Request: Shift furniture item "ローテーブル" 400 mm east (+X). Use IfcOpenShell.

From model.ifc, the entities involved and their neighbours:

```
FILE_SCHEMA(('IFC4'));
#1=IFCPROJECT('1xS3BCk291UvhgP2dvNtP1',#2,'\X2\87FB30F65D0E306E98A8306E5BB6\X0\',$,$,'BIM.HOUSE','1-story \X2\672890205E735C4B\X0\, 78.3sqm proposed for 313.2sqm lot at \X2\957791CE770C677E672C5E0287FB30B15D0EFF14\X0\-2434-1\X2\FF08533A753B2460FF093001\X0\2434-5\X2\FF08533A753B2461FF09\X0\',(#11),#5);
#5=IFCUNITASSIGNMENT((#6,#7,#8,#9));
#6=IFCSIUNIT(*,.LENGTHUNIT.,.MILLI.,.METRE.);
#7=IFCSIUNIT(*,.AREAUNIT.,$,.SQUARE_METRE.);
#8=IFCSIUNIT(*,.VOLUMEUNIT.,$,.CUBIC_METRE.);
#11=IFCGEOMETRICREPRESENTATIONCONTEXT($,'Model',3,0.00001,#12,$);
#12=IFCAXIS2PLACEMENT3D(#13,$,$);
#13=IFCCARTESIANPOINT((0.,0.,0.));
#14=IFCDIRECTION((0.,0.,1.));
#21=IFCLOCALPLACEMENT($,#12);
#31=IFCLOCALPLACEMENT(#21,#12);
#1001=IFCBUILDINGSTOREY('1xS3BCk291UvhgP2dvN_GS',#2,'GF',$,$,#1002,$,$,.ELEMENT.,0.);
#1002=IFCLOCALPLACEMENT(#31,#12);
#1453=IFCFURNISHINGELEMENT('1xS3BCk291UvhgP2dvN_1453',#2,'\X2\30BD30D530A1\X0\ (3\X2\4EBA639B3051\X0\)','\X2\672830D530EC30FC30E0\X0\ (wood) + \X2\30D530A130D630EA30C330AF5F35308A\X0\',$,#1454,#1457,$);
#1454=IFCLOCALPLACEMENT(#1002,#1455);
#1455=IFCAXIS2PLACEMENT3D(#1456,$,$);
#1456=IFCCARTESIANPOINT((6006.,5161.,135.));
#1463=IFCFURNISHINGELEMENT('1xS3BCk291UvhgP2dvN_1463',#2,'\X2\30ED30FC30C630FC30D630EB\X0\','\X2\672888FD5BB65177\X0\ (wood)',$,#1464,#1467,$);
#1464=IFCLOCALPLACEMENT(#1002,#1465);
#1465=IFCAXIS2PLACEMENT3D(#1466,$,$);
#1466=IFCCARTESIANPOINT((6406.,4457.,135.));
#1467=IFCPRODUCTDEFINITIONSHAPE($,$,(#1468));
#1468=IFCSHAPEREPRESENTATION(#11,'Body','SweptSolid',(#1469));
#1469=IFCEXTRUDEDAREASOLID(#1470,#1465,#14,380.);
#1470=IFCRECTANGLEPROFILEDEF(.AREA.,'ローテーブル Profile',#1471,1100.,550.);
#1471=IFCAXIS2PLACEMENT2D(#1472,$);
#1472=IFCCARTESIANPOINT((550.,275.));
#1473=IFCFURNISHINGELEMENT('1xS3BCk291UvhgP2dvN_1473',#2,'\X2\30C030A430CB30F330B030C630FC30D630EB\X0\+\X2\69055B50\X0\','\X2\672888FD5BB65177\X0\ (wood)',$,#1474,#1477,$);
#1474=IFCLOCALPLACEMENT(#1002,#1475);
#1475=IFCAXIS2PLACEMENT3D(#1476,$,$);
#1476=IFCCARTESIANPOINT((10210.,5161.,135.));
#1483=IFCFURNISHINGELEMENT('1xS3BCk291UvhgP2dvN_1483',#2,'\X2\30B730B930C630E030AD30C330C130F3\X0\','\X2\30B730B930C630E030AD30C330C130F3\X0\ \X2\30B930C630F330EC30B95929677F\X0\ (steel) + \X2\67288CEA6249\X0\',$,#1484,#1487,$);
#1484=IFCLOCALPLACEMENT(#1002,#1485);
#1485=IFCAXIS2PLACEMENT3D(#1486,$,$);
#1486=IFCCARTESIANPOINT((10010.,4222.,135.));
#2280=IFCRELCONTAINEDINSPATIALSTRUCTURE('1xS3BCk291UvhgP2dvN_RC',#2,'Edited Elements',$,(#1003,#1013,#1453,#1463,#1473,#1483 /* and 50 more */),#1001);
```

```python
import ifcopenshell
import ifcopenshell.api.geometry
import ifcopenshell.util.placement
import ifcopenshell.util.unit

model = ifcopenshell.open("model.ifc")
unit_scale = ifcopenshell.util.unit.calculate_unit_scale(model)

item = model.by_guid("1xS3BCk291UvhgP2dvN_1463")
matrix = ifcopenshell.util.placement.get_local_placement(item.ObjectPlacement)
matrix[0, 3] += 0.4 / unit_scale
ifcopenshell.api.geometry.edit_object_placement(model, product=item, matrix=matrix, is_si=False)

print(ifcopenshell.util.placement.get_local_placement(item.ObjectPlacement).round(3) + 0.0)

model.write("model_v2.ifc")
```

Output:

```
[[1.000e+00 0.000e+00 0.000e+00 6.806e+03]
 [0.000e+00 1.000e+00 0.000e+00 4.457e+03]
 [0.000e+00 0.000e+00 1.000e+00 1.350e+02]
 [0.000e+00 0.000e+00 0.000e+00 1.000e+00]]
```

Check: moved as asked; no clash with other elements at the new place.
